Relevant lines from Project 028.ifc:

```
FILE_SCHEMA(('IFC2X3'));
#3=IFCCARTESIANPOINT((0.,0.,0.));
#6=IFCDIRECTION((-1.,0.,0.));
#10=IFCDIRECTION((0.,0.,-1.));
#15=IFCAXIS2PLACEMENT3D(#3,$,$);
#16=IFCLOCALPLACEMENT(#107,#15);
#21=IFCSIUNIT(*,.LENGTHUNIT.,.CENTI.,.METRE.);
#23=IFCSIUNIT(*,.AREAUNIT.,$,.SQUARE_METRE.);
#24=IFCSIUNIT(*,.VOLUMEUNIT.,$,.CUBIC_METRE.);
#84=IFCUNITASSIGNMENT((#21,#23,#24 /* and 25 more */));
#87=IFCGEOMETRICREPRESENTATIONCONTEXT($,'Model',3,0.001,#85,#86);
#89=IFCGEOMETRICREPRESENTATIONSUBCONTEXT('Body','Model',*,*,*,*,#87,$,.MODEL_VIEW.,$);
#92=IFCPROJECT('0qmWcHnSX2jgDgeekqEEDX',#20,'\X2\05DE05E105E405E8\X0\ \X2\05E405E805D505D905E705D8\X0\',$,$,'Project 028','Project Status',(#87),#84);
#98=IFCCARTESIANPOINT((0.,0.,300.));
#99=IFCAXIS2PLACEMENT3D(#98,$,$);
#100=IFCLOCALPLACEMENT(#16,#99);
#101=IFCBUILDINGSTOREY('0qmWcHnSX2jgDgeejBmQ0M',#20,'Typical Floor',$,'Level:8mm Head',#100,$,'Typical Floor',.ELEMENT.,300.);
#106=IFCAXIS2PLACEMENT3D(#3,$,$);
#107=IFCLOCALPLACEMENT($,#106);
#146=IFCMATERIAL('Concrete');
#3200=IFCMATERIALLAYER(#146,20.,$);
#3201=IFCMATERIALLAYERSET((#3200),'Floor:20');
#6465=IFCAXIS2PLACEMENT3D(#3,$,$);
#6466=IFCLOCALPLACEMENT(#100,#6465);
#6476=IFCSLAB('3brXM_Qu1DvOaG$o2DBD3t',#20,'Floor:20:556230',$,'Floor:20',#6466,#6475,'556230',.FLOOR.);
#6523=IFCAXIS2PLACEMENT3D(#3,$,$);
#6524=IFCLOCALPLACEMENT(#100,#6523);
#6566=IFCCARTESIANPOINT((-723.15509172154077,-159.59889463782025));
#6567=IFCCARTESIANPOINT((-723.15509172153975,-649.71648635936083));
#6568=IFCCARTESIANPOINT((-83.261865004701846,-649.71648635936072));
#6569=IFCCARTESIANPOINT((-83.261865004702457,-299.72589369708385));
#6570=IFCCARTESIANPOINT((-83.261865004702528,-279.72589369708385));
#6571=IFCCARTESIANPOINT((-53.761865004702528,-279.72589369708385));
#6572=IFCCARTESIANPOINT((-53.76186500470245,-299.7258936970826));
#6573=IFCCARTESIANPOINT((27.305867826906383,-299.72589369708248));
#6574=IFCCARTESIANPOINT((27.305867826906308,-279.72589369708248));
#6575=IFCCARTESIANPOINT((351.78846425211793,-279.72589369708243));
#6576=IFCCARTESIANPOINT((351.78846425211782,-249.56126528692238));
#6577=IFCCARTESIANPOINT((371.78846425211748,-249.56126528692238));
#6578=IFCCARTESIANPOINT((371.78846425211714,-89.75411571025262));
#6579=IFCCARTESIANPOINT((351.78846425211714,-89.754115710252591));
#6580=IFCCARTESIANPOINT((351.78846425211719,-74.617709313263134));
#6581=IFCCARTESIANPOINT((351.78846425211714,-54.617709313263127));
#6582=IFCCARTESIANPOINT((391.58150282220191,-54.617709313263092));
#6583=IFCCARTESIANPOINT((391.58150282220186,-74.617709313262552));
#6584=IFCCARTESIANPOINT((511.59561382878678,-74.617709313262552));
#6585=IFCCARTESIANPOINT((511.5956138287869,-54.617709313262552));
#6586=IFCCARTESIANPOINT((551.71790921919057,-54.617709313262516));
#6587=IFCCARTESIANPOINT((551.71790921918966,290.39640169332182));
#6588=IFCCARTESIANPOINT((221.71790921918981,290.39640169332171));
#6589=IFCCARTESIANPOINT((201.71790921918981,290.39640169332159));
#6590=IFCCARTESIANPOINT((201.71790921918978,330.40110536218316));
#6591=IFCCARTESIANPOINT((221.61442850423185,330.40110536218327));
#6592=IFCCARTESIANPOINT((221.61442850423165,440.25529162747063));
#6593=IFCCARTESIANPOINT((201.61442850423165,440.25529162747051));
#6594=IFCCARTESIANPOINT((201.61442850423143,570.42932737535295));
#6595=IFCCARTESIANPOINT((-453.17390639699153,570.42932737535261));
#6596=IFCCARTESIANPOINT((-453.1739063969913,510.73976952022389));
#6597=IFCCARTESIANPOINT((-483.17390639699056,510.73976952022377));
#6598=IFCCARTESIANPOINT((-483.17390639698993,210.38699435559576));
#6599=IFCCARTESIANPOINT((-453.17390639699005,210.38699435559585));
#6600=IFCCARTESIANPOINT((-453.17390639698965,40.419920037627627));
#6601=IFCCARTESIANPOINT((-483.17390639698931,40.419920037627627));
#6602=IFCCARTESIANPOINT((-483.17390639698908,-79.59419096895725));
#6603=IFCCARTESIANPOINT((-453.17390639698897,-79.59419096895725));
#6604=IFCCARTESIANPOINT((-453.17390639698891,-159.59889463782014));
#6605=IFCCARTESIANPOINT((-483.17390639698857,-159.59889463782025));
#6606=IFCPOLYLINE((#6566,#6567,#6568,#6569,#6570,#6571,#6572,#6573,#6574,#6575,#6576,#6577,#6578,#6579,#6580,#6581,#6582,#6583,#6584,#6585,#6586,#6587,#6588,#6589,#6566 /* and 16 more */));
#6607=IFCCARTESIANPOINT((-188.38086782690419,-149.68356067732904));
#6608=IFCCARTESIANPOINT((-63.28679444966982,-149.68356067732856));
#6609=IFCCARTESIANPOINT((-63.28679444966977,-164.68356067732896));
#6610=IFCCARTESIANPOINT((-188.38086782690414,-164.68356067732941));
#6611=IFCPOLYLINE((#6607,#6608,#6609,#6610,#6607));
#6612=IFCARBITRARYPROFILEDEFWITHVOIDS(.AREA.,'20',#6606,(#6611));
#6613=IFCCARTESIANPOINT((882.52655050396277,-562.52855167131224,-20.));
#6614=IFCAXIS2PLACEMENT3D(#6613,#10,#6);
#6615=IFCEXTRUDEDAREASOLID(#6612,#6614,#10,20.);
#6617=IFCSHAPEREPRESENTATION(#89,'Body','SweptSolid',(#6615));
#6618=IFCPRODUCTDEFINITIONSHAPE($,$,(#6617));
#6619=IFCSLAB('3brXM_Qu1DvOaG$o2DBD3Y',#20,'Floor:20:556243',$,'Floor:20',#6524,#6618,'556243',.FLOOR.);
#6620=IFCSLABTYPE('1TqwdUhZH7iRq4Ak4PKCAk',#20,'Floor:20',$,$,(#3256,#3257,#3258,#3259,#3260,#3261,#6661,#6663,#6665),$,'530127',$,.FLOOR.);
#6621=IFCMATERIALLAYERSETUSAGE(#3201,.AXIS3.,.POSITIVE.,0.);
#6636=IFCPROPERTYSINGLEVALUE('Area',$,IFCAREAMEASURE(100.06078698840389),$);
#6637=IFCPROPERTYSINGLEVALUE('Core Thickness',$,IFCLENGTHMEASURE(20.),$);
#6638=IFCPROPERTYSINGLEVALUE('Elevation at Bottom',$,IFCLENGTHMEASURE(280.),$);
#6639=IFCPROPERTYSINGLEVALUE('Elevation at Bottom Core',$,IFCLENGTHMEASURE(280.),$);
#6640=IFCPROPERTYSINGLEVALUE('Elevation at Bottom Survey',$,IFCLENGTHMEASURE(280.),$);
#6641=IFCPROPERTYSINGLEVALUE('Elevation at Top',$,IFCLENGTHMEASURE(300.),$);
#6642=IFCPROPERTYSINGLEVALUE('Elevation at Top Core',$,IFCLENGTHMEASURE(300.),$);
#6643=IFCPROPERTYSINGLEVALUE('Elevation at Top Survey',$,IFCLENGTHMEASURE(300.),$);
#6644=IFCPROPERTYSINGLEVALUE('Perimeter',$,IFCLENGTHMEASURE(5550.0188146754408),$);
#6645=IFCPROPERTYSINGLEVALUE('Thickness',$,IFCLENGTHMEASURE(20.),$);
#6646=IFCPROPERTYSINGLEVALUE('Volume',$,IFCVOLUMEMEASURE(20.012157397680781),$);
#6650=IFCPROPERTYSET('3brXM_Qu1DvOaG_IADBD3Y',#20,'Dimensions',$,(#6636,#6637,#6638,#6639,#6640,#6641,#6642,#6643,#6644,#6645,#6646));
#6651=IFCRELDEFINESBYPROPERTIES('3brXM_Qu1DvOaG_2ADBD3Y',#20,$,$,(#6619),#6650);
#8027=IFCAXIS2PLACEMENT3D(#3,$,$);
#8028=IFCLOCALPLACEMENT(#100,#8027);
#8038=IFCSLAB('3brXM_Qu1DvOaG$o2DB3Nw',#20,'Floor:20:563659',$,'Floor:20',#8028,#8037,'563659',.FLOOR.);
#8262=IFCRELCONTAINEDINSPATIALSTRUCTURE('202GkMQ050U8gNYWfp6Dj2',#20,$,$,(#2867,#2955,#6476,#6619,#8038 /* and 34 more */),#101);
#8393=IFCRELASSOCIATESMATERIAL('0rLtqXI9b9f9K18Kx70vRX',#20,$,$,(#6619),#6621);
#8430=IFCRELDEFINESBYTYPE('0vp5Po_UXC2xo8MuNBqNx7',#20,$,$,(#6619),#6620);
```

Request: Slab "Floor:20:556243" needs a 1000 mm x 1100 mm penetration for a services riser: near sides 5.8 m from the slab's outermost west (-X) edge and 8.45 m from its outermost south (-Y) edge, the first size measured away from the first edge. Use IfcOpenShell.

```python
import numpy as np
import ifcopenshell
import ifcopenshell.api.feature
import ifcopenshell.api.geometry
import ifcopenshell.api.pset
import ifcopenshell.api.root
import ifcopenshell.geom
import ifcopenshell.util.element
import ifcopenshell.util.placement
import ifcopenshell.util.representation
import ifcopenshell.util.shape
import ifcopenshell.util.unit

model = ifcopenshell.open("Project 028.ifc")
unit_scale = ifcopenshell.util.unit.calculate_unit_scale(model)
area_scale = ifcopenshell.util.unit.calculate_unit_scale(model, "AREAUNIT")
volume_scale = ifcopenshell.util.unit.calculate_unit_scale(model, "VOLUMEUNIT")
settings = ifcopenshell.geom.settings()


def volume(element):
    """Net volume in cubic metres, openings subtracted."""
    shape = ifcopenshell.geom.create_shape(settings, element)
    return ifcopenshell.util.shape.get_volume(shape.geometry)


slab = model.by_guid("3brXM_Qu1DvOaG$o2DBD3Y")
before = volume(slab)

# Extent in the slab's own axes, in metres. The edges named are its -X and -Y sides.
slab_shape = ifcopenshell.geom.create_shape(settings, slab)
vertices = ifcopenshell.util.shape.get_vertices(slab_shape.geometry)
x_min, y_min, bottom = vertices.min(axis=0)
top = vertices[:, 2].max()

opening = ifcopenshell.api.root.create_entity(model, ifc_class="IfcOpeningElement", name="Services riser opening")
context = ifcopenshell.util.representation.get_context(model, "Model", "Body", "MODEL_VIEW")
width, depth = 1, 1.1
outline = [(0.0, 0.0), (width, 0.0), (width, depth), (0.0, depth), (0.0, 0.0)]
# Overshoot both faces by 50 mm so the cut is clean.
shape = ifcopenshell.api.geometry.add_slab_representation(
    model, context=context, depth=top - bottom + 0.1, polyline=outline
)
ifcopenshell.api.geometry.assign_representation(model, product=opening, representation=shape)

matrix = ifcopenshell.util.placement.get_local_placement(slab.ObjectPlacement)
matrix[:, 3] = matrix @ np.append(np.array([x_min + 5.8, y_min + 8.45, bottom - 0.05]) / unit_scale, 1.0)
ifcopenshell.api.geometry.edit_object_placement(model, product=opening, matrix=matrix, is_si=False)
ifcopenshell.api.feature.add_feature(model, feature=opening, element=slab)

after = volume(slab)

# Update the slab's stored quantities.
pset = model.by_id(ifcopenshell.util.element.get_pset(slab, "Dimensions", should_inherit=False)["id"])
ifcopenshell.api.pset.edit_pset(model, pset=pset, properties={
    "Area": model.create_entity("IfcAreaMeasure", after / (top - bottom) / area_scale),
    "Volume": model.create_entity("IfcVolumeMeasure", after / volume_scale),
})

print(f"slab volume {before:.3f} -> {after:.3f} m3")

model.write("Project 028_updated.ifc")
```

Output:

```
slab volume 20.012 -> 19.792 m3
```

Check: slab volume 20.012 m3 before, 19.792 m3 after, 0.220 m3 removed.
